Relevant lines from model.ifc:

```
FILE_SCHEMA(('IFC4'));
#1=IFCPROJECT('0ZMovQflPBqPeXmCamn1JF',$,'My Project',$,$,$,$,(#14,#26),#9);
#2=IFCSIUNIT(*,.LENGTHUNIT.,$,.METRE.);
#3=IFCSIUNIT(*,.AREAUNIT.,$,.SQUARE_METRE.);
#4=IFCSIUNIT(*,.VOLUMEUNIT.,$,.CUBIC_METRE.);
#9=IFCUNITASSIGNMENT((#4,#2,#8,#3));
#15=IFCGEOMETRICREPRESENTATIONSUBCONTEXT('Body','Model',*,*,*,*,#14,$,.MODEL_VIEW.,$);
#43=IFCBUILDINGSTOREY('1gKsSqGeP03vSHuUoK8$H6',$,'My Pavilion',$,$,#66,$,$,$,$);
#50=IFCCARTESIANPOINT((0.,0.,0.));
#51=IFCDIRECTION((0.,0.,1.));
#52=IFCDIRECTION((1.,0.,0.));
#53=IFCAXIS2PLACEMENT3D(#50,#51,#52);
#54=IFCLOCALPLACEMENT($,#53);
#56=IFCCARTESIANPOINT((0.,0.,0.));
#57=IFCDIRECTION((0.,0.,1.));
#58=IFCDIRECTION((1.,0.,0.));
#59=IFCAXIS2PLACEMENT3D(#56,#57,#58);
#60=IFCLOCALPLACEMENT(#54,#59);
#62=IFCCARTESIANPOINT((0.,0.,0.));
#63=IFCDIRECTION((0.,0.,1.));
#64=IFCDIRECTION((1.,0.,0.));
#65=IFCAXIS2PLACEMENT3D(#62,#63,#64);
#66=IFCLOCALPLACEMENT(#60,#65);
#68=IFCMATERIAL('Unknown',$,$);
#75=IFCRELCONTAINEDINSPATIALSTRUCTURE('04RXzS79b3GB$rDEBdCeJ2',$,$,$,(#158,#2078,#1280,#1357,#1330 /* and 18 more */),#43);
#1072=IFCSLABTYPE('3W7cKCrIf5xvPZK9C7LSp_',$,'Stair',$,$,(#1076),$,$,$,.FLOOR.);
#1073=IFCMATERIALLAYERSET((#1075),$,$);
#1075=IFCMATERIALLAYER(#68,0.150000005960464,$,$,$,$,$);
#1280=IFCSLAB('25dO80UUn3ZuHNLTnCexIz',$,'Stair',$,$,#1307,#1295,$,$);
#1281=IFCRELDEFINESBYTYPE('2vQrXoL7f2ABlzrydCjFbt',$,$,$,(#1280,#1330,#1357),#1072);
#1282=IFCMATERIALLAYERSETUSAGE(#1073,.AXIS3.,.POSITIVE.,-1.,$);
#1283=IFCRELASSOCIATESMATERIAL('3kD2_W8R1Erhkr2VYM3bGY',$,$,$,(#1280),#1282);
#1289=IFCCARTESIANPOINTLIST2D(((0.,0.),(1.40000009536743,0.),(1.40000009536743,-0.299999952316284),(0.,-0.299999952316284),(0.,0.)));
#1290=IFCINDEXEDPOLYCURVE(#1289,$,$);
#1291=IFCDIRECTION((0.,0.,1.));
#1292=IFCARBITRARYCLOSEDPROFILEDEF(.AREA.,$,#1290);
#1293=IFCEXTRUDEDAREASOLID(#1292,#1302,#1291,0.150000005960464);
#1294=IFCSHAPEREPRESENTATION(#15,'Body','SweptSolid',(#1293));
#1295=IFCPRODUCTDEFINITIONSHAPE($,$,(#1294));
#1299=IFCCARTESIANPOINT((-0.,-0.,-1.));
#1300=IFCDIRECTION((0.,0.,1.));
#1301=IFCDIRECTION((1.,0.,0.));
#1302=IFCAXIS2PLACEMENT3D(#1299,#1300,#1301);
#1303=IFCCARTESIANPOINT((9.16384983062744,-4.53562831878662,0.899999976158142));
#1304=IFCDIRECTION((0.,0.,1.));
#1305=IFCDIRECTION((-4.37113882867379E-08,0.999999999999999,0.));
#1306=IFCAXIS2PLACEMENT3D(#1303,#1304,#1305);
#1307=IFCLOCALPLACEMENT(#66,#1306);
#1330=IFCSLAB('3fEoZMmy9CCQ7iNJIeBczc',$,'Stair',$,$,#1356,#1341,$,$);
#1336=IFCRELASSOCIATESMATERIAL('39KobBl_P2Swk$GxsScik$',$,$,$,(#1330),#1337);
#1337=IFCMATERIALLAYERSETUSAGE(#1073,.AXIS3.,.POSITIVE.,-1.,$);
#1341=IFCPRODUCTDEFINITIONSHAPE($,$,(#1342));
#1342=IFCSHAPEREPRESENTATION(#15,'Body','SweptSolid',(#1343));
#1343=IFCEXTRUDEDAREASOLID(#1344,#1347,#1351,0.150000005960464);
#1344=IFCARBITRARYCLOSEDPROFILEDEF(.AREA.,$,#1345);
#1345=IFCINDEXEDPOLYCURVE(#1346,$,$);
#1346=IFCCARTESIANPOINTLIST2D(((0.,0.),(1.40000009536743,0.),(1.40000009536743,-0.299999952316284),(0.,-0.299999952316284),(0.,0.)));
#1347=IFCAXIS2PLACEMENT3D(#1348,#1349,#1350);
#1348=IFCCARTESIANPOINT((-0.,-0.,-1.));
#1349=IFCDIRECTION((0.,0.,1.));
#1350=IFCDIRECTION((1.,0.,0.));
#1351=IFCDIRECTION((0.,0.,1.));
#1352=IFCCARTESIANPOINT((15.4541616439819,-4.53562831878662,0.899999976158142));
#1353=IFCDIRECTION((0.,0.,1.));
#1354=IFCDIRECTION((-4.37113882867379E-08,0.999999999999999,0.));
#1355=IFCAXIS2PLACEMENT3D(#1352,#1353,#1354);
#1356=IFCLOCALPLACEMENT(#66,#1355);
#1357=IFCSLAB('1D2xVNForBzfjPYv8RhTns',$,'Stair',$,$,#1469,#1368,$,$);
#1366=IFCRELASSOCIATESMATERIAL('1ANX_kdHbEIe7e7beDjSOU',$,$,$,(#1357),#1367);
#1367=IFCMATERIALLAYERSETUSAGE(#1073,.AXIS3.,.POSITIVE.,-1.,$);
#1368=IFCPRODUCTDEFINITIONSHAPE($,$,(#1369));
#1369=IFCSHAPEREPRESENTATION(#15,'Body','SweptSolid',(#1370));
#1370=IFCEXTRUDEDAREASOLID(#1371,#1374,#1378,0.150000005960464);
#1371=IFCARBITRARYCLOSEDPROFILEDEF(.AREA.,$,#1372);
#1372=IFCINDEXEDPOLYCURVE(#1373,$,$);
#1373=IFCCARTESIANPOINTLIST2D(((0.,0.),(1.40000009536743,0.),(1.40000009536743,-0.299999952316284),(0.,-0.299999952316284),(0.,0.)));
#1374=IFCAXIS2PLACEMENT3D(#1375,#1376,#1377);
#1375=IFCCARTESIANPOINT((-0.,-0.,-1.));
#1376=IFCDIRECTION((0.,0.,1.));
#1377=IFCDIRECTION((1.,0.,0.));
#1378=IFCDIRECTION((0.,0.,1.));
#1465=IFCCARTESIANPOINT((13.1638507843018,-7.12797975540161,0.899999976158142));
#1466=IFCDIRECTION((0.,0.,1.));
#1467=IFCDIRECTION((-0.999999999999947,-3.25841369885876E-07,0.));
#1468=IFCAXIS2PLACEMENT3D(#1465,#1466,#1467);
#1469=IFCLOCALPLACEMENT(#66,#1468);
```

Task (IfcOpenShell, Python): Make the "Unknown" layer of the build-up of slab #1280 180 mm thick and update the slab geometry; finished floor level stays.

```python
import ifcopenshell
import ifcopenshell.util.element
import ifcopenshell.util.representation
import ifcopenshell.util.unit

model = ifcopenshell.open("model.ifc")
unit_scale = ifcopenshell.util.unit.calculate_unit_scale(model)

layer_set = model.by_id(1073)
layer = next(l for l in layer_set.MaterialLayers if l.Material and l.Material.Name == "Unknown")
change = 0.18 / unit_scale - layer.LayerThickness
layer.LayerThickness += change

# The layer set is shared, so every slab that uses it gets the new thickness.
slabs = [e for e in ifcopenshell.util.element.get_elements_by_material(model, layer_set) if e.is_a("IfcSlab")]
for slab in sorted(slabs, key=lambda e: e.id()):
    body = ifcopenshell.util.representation.get_representation(slab, "Model", "Body")
    solid = body.Items[0]
    old_depth = solid.Depth
    solid.Depth += change
    # Extruded upwards: lower the start of the extrusion so the top stays.
    x, y, z = solid.Position.Location.Coordinates
    solid.Position.Location = model.createIfcCartesianPoint((x, y, z - change))
    print(slab.id(), f"{old_depth:g} -> {solid.Depth:g}")

# The layers are counted up from the underside, which has moved.
for usage in {ifcopenshell.util.element.get_material(slab) for slab in slabs}:
    usage.OffsetFromReferenceLine -= change

model.write("model_edited.ifc")
```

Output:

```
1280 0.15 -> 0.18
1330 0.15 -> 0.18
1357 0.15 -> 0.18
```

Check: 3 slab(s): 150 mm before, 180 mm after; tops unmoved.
